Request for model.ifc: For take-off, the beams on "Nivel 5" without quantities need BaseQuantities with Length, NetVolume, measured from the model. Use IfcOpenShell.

First a look at what the model holds.

```python
import ifcopenshell
import ifcopenshell.util.element
import ifcopenshell.util.unit

model = ifcopenshell.open("model.ifc")
print(model.schema)
for unit_type in ("LENGTHUNIT", "AREAUNIT", "VOLUMEUNIT"):
    print(unit_type, ifcopenshell.util.unit.calculate_unit_scale(model, unit_type))
storey = next(s for s in model.by_type("IfcBuildingStorey") if s.Name == "Nivel 5")
beams = [e for e in ifcopenshell.util.element.get_decomposition(storey) if e.is_a("IfcBeam")]
for e in sorted(beams, key=lambda e: e.id()):
    print(e.id(), e.is_a(), e.Name, list(ifcopenshell.util.element.get_psets(e, qtos_only=True)), sep=" | ")
```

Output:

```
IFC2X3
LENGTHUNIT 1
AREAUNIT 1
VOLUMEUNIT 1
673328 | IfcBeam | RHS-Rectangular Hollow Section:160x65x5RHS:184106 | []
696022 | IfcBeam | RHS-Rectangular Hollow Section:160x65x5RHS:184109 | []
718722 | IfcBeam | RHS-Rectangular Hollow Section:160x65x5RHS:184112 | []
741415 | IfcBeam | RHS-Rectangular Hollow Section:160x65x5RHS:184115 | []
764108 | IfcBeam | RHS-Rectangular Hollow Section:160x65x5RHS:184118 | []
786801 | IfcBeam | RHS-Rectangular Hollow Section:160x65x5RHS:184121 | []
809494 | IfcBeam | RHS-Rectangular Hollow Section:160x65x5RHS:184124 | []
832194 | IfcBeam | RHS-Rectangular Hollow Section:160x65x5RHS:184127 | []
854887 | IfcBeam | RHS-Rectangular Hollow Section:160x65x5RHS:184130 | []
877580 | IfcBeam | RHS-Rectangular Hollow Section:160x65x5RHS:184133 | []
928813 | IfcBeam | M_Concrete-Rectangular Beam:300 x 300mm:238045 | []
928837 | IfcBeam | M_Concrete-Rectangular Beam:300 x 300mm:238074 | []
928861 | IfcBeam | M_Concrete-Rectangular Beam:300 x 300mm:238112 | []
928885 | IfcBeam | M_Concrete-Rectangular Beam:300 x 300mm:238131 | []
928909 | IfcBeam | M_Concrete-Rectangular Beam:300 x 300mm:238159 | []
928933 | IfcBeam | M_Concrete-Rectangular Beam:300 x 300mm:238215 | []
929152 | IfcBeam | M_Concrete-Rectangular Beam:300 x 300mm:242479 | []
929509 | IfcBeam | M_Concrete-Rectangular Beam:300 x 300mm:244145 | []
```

```python
import ifcopenshell
import ifcopenshell.api.pset
import ifcopenshell.geom
import ifcopenshell.util.element
import ifcopenshell.util.shape
import ifcopenshell.util.unit

model = ifcopenshell.open("model.ifc")
unit_scale = ifcopenshell.util.unit.calculate_unit_scale(model)
volume_scale = ifcopenshell.util.unit.calculate_unit_scale(model, "VOLUMEUNIT")
settings = ifcopenshell.geom.settings()

storey = next(s for s in model.by_type("IfcBuildingStorey") if s.Name == "Nivel 5")
beams = [e for e in ifcopenshell.util.element.get_decomposition(storey) if e.is_a("IfcBeam")]

for e in sorted(beams, key=lambda e: e.id()):
    if ifcopenshell.util.element.get_psets(e, qtos_only=True, should_inherit=False):
        continue
    # Geometry comes back in metres, in the element's own axes.
    shape = ifcopenshell.geom.create_shape(settings, e)
    values = {
        "Length": ifcopenshell.util.shape.get_max_xyz(shape.geometry) / unit_scale,
        "NetVolume": ifcopenshell.util.shape.get_volume(shape.geometry) / volume_scale,
    }
    qto = ifcopenshell.api.pset.add_qto(model, product=e, name="BaseQuantities")
    ifcopenshell.api.pset.edit_qto(model, qto=qto, properties=values)
    print(e.id(), {k: round(v, 3) for k, v in values.items()})

model.write("model-out.ifc")
```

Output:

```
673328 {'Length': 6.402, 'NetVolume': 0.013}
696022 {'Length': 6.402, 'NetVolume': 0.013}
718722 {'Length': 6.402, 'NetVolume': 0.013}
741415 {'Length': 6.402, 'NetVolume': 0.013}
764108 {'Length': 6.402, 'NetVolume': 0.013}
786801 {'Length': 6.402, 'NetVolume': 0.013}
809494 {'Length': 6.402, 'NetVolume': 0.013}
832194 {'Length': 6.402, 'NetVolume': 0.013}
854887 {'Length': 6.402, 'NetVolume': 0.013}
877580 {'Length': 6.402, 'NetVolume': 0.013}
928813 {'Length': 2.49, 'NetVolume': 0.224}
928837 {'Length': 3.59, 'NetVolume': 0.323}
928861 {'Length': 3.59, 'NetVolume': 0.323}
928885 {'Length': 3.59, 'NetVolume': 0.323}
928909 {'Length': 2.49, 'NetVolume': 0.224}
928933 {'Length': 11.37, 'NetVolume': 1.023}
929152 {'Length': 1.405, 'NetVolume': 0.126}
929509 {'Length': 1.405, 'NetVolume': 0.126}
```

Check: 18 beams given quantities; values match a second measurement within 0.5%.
